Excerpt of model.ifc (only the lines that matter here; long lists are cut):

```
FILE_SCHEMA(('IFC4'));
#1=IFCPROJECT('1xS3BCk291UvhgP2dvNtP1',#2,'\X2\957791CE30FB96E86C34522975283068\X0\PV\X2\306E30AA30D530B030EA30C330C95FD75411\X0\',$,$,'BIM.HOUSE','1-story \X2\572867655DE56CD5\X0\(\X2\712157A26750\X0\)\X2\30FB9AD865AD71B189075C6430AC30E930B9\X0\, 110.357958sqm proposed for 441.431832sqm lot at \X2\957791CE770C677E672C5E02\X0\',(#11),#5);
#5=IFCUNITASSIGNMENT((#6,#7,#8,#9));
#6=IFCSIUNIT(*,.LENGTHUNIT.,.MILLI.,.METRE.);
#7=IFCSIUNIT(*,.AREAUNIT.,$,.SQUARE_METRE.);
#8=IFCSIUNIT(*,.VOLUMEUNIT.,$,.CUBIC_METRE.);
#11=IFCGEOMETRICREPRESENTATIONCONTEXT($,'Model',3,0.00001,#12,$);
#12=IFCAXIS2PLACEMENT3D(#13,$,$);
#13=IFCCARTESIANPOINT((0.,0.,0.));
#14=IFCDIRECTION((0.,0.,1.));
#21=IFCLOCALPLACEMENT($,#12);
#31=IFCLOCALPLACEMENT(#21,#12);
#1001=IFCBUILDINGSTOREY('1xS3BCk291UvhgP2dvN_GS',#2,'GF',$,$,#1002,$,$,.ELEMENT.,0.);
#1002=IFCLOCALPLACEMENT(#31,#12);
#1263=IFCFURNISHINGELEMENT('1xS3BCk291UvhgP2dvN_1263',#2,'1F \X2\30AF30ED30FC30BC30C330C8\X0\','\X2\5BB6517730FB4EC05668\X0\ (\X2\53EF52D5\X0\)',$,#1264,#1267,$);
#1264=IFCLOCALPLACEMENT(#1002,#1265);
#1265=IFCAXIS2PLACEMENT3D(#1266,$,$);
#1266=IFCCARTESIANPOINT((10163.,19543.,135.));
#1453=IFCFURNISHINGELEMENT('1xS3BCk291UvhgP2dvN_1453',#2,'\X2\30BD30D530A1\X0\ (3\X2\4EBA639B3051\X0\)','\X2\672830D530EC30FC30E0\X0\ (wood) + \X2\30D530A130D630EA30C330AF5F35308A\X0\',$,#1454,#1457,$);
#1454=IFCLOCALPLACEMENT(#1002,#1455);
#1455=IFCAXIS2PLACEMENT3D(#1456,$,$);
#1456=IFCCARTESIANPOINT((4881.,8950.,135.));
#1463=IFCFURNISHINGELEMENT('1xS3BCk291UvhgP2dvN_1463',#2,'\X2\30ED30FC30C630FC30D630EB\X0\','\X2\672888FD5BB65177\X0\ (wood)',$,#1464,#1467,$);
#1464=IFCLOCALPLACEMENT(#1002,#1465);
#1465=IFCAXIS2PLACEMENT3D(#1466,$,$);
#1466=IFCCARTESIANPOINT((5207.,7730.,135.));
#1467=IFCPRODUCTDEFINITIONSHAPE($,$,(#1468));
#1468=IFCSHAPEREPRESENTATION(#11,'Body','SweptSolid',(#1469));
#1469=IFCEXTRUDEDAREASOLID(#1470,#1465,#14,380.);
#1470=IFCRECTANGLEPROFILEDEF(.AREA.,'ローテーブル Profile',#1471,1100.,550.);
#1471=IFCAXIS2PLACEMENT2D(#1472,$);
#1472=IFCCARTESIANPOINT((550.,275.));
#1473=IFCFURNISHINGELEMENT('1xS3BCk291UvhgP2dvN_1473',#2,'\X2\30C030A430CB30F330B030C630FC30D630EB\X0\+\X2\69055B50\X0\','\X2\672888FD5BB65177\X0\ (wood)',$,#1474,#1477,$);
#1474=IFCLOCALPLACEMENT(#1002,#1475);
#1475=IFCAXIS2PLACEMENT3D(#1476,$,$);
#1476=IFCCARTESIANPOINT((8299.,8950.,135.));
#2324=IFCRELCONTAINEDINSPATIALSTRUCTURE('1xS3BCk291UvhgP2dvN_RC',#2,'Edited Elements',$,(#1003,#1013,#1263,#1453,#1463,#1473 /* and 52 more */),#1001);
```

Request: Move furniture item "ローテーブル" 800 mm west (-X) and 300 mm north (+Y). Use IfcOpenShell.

```python
import ifcopenshell
import ifcopenshell.api.geometry
import ifcopenshell.util.placement

model = ifcopenshell.open("model.ifc")

item = model.by_guid("1xS3BCk291UvhgP2dvN_1463")
matrix = ifcopenshell.util.placement.get_local_placement(item.ObjectPlacement)
matrix[0, 3] -= 800.0
matrix[1, 3] += 300.0
ifcopenshell.api.geometry.edit_object_placement(model, product=item, matrix=matrix, is_si=False)

print(ifcopenshell.util.placement.get_local_placement(item.ObjectPlacement).round(3) + 0.0)

model.write("model_v2.ifc")
```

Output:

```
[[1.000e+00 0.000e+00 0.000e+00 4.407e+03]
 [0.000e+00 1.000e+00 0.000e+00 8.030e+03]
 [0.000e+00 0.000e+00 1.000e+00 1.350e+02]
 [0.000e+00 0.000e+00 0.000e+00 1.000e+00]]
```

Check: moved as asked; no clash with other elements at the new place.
